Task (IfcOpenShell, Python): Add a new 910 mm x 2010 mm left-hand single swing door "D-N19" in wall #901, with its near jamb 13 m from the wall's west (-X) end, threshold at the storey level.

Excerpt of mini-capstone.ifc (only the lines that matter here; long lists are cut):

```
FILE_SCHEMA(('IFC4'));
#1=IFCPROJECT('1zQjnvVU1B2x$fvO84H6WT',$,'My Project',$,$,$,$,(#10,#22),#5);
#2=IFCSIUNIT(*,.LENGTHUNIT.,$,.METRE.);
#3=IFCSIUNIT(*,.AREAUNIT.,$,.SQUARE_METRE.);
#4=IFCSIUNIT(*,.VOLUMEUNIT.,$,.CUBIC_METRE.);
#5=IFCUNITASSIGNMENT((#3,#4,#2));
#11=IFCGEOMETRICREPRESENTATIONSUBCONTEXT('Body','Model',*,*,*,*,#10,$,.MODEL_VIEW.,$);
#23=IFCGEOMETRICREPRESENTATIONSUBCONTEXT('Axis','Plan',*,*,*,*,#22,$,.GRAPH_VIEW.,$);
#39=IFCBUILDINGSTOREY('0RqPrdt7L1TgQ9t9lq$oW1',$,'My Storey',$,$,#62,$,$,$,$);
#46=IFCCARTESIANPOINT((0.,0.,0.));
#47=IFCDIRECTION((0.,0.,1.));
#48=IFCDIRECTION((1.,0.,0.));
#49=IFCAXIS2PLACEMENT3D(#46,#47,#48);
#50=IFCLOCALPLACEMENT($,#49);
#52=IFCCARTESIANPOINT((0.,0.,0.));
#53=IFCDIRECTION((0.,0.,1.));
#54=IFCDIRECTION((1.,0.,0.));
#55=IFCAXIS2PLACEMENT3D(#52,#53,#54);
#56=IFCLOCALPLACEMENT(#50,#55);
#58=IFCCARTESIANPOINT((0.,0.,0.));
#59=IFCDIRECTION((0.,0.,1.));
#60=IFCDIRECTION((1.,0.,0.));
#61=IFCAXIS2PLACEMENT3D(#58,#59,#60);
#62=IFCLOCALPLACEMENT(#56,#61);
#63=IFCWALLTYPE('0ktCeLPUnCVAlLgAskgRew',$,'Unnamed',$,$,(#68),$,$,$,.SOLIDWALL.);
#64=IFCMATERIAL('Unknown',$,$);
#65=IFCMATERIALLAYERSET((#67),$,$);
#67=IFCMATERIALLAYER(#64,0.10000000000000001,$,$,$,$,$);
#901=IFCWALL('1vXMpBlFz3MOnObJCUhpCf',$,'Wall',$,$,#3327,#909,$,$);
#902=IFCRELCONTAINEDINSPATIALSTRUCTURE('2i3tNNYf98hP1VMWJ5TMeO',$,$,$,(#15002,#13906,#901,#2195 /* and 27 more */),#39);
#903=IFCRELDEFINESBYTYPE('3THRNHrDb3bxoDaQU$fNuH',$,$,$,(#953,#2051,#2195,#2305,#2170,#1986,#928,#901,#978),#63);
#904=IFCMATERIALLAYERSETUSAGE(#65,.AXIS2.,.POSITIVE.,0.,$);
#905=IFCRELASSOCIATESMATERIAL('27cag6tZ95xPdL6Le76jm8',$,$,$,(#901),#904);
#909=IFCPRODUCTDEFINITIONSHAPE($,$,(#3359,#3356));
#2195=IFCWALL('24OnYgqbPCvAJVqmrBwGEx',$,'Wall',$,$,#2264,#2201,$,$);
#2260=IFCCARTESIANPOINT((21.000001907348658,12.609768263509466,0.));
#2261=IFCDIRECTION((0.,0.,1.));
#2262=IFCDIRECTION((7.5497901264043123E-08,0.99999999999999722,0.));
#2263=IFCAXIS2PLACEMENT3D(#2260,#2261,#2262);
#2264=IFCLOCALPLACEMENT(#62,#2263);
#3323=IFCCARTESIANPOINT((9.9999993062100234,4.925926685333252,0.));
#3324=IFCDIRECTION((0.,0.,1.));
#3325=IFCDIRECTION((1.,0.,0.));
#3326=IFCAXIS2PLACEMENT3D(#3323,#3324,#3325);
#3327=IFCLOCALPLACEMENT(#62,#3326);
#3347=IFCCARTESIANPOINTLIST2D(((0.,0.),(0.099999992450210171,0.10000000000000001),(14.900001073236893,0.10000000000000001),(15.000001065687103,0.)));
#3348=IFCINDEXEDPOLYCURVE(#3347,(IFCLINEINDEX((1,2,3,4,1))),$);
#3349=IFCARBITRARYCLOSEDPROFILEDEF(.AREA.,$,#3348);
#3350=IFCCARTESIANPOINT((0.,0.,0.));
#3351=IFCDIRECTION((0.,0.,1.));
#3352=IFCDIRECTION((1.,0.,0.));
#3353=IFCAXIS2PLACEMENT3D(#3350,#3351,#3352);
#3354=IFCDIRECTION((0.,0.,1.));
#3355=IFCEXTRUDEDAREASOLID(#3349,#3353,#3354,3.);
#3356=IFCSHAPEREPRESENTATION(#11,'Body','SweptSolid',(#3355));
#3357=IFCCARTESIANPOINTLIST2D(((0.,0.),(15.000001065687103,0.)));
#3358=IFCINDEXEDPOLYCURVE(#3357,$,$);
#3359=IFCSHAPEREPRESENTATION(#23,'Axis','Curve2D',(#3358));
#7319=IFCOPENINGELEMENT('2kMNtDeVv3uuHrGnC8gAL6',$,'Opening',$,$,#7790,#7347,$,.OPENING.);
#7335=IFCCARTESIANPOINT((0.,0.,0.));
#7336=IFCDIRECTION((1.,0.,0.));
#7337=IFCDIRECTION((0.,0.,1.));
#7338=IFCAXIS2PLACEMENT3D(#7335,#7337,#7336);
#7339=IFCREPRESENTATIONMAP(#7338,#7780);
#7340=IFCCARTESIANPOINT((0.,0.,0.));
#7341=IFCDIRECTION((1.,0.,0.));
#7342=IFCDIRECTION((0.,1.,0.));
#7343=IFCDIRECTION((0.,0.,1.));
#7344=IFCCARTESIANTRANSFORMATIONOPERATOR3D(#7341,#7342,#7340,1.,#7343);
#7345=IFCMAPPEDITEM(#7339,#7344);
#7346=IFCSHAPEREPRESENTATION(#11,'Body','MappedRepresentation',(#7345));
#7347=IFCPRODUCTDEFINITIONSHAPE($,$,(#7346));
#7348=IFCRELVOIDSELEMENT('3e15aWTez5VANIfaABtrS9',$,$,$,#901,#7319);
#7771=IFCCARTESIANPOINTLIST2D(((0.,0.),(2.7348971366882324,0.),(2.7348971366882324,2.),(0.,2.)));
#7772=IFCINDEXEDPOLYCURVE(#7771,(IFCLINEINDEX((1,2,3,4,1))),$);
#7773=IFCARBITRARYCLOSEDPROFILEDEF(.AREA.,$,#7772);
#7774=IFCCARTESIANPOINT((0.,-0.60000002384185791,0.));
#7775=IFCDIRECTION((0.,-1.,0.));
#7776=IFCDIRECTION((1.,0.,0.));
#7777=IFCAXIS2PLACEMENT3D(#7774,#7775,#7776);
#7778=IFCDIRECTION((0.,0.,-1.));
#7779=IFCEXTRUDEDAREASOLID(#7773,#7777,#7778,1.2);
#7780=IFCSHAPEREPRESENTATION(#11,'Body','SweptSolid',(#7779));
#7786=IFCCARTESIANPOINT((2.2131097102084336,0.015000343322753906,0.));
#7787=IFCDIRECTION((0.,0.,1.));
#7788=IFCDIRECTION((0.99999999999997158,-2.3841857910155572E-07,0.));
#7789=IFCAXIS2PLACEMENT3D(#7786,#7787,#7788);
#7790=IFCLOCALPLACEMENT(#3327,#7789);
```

```python
import numpy as np
import ifcopenshell
import ifcopenshell.api.feature
import ifcopenshell.api.geometry
import ifcopenshell.api.root
import ifcopenshell.api.spatial
import ifcopenshell.geom
import ifcopenshell.util.element
import ifcopenshell.util.placement
import ifcopenshell.util.representation
import ifcopenshell.util.shape
import ifcopenshell.util.unit

model = ifcopenshell.open("mini-capstone.ifc")
unit_scale = ifcopenshell.util.unit.calculate_unit_scale(model)
settings = ifcopenshell.geom.settings()


def volume(element):
    """Net volume in cubic metres, openings subtracted."""
    shape = ifcopenshell.geom.create_shape(settings, element)
    return ifcopenshell.util.shape.get_volume(shape.geometry)


wall = model.by_id(901)
storey = ifcopenshell.util.element.get_container(wall, ifc_class="IfcBuildingStorey")
context = ifcopenshell.util.representation.get_context(model, "Model", "Body", "MODEL_VIEW")
before = volume(wall)

width, height, from_end, sill = 0.91, 2.01, 13, 0.0  # metres

# The wall runs along its own X axis, and the end named is its -X end.
wall_shape = ifcopenshell.geom.create_shape(settings, wall)
x, y, z = ifcopenshell.util.shape.get_vertices(wall_shape.geometry).T
start = x.min() + from_end
face, thickness = float(y.min()), float(y.max() - y.min())
wall_matrix = ifcopenshell.util.placement.get_local_placement(wall.ObjectPlacement)
level = ifcopenshell.util.placement.get_local_placement(storey.ObjectPlacement)[2, 3]


def in_wall(x, y):
    """Placement at x, y metres in the wall's axes, at sill height."""
    matrix = wall_matrix.copy()
    matrix[:, 3] = wall_matrix @ np.array([x / unit_scale, y / unit_scale, 0.0, 1.0])
    matrix[2, 3] = level + sill / unit_scale
    return matrix


# Opening: a box that overshoots both wall faces by 50 mm.
opening = ifcopenshell.api.root.create_entity(model, ifc_class="IfcOpeningElement", predefined_type="OPENING")
box = ifcopenshell.api.geometry.add_wall_representation(
    model, context=context, length=width, height=height, thickness=thickness + 0.1
)
ifcopenshell.api.geometry.assign_representation(model, product=opening, representation=box)
ifcopenshell.api.geometry.edit_object_placement(model, product=opening, matrix=in_wall(start, face - 0.05), is_si=False)
ifcopenshell.api.feature.add_feature(model, feature=opening, element=wall)

door = ifcopenshell.api.root.create_entity(model, ifc_class="IfcDoor", name="D-N19", predefined_type="DOOR")
door.OverallWidth, door.OverallHeight = width / unit_scale, height / unit_scale
door.OperationType = "SINGLE_SWING_LEFT"
body = ifcopenshell.api.geometry.add_door_representation(
    model,
    context=context,
    overall_width=door.OverallWidth,
    overall_height=door.OverallHeight,
    operation_type="SINGLE_SWING_LEFT",
    lining_properties={"LiningDepth": thickness / unit_scale, "ThresholdDepth": thickness / unit_scale},
)
ifcopenshell.api.geometry.assign_representation(model, product=door, representation=body)
ifcopenshell.api.spatial.assign_container(model, products=[door], relating_structure=storey)
ifcopenshell.api.feature.add_filling(model, opening=opening, element=door)

# The lining spans the wall, so the door starts at the wall face.
ifcopenshell.api.geometry.edit_object_placement(model, product=door, matrix=in_wall(start, face), is_si=False)

after = volume(wall)

print(f"wall volume {before:.3f} -> {after:.3f} m3")

model.write("mini-capstone_edited.ifc")
```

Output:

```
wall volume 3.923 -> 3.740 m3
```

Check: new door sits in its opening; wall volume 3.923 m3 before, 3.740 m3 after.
